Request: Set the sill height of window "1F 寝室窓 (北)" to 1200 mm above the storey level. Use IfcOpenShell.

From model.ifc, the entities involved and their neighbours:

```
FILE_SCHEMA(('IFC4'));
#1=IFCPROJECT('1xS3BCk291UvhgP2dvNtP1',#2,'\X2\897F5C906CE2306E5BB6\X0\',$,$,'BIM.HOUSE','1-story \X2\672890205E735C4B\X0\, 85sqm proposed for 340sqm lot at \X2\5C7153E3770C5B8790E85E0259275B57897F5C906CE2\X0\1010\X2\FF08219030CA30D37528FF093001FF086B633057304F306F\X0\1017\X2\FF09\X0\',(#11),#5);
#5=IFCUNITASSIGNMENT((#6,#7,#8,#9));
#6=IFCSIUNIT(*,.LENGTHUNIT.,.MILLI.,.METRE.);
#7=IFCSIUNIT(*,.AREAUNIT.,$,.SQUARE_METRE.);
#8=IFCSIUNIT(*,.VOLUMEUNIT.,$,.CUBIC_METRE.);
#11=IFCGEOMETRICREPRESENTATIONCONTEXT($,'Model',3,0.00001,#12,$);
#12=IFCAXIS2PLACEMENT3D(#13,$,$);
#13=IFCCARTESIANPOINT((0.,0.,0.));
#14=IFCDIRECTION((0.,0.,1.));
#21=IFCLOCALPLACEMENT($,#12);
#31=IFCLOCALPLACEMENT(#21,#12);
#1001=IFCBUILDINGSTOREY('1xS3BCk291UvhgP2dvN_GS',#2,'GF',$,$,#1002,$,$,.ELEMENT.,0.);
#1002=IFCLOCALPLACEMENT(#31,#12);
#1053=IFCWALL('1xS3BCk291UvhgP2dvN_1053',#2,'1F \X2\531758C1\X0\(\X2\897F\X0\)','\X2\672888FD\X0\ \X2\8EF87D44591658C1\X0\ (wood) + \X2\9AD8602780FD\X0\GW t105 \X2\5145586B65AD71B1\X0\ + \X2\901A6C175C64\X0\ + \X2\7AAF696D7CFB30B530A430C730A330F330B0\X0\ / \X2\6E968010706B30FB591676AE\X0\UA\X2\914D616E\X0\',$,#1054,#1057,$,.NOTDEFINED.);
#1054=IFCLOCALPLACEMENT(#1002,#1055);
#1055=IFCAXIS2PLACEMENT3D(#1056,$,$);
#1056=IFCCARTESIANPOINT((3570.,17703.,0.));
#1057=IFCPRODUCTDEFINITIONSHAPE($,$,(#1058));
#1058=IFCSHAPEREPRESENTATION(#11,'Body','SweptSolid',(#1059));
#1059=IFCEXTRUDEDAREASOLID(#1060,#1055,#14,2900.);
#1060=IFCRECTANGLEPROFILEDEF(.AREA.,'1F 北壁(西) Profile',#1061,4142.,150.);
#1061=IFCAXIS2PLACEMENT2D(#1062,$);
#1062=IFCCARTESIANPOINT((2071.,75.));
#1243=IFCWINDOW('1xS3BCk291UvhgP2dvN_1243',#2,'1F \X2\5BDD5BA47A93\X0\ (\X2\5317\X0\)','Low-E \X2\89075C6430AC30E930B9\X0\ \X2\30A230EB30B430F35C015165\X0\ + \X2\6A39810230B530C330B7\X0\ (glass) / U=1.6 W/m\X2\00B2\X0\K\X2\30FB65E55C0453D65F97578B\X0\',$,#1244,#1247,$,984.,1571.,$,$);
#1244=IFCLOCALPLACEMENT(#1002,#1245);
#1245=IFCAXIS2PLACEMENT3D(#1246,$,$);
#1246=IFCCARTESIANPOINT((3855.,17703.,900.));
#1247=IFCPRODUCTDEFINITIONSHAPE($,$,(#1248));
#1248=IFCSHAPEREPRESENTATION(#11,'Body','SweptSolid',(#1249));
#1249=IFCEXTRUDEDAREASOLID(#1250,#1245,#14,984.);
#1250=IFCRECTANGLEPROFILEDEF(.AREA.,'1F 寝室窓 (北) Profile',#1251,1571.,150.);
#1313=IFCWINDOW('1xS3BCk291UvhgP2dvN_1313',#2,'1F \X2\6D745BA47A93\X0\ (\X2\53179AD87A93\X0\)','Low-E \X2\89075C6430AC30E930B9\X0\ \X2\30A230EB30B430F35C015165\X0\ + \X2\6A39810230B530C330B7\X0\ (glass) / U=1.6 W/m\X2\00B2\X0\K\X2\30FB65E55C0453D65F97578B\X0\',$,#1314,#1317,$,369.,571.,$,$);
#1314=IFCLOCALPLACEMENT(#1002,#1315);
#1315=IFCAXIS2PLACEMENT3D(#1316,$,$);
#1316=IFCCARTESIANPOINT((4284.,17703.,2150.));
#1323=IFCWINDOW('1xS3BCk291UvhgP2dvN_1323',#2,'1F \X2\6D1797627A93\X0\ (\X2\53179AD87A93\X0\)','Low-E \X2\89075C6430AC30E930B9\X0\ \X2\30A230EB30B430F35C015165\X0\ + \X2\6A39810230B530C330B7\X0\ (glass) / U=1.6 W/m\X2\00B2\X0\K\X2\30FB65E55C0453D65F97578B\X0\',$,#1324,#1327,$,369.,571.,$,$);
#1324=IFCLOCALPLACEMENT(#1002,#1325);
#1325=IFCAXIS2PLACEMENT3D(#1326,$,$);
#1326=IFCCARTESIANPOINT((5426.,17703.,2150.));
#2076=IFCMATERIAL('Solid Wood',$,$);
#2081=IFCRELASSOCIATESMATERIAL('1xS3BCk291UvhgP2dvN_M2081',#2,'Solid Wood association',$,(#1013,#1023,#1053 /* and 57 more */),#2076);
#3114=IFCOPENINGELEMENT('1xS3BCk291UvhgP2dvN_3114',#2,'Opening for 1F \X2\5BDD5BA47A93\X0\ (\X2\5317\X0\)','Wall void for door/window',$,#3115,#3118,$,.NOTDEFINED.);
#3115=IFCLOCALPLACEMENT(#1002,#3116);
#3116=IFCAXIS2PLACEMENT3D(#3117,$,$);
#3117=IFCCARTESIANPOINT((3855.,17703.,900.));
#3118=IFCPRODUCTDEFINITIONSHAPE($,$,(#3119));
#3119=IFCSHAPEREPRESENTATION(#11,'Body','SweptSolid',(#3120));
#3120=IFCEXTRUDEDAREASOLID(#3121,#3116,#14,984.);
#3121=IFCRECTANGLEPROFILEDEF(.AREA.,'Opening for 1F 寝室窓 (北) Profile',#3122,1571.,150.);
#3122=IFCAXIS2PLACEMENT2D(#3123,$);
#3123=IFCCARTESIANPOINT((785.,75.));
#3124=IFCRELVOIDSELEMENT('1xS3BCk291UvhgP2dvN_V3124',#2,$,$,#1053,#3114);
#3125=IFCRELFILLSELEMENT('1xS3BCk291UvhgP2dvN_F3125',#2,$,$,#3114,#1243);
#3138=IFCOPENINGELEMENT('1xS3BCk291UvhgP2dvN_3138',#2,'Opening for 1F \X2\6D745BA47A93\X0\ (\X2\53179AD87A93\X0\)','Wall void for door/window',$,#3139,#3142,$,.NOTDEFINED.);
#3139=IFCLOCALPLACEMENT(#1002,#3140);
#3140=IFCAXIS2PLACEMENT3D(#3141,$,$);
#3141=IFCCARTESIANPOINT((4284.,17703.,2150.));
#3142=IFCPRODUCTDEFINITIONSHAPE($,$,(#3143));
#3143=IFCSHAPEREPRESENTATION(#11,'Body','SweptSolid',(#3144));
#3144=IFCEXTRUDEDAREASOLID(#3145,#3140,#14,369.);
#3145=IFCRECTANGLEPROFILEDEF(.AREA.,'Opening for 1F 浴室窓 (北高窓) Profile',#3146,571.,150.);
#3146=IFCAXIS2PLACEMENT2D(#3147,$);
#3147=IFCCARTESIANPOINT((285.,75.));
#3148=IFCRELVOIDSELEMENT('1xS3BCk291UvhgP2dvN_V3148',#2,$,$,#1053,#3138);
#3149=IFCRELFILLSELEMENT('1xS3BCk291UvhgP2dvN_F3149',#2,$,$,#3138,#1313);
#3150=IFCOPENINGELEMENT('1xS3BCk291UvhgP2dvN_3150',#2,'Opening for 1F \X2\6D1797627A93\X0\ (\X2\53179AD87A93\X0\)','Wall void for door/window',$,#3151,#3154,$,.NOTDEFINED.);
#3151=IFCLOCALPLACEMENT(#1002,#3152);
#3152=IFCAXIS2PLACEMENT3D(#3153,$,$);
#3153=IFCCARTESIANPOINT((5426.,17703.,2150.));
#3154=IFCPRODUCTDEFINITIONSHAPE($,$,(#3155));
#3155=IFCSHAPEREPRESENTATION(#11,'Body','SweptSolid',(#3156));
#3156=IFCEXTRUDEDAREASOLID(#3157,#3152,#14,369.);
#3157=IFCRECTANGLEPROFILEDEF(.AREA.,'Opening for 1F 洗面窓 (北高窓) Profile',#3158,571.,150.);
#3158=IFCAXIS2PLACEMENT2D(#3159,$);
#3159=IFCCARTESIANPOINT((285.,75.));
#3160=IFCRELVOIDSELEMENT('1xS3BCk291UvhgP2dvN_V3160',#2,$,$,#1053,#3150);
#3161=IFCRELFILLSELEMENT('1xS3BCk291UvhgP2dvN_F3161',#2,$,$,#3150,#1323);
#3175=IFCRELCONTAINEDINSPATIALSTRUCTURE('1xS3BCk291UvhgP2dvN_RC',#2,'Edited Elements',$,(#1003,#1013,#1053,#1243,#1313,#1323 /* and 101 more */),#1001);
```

```python
import numpy as np
import ifcopenshell
import ifcopenshell.api.geometry
import ifcopenshell.geom
import ifcopenshell.util.element
import ifcopenshell.util.placement
import ifcopenshell.util.shape
import ifcopenshell.util.unit

model = ifcopenshell.open("model.ifc")
unit_scale = ifcopenshell.util.unit.calculate_unit_scale(model)

window = model.by_guid("1xS3BCk291UvhgP2dvN_1243")
opening = window.FillsVoids[0].RelatingOpeningElement
storey = ifcopenshell.util.element.get_container(window, ifc_class="IfcBuildingStorey")
level = ifcopenshell.util.placement.get_local_placement(storey.ObjectPlacement)[2, 3]

# The opening's origin need not be at the sill, so measure its lowest point.
shape = ifcopenshell.geom.create_shape(ifcopenshell.geom.settings(), opening)
bottom = ifcopenshell.util.shape.get_shape_bottom_elevation(shape, shape.geometry) / unit_scale
dz = level + 1200.0 - bottom

shift = np.array([0.0, 0.0, dz])
# The window is not placed relative to its opening, so move both.
for product in (opening, window):
    matrix = ifcopenshell.util.placement.get_local_placement(product.ObjectPlacement)
    matrix[:3, 3] += shift
    ifcopenshell.api.geometry.edit_object_placement(model, product=product, matrix=matrix, is_si=False)

print(f"moved by {dz * unit_scale:+.3f} m")

model.write("model_edited.ifc")
```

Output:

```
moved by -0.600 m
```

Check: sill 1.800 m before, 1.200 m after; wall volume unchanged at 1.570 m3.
